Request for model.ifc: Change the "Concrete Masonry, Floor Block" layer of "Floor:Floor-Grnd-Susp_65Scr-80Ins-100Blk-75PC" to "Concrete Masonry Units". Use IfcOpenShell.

First a look at what the model holds.

```python
import ifcopenshell
import ifcopenshell.util.element

model = ifcopenshell.open("model.ifc")
print(model.schema)
for layer_set in model.by_type("IfcMaterialLayerSet"):
    if layer_set.LayerSetName == "Floor:Floor-Grnd-Susp_65Scr-80Ins-100Blk-75PC":
        for layer in layer_set.MaterialLayers:
            print(layer.id(), layer.Material and layer.Material.Name, layer.LayerThickness, sep=" | ")
        print(len(ifcopenshell.util.element.get_elements_by_material(model, layer_set)), "elements and types use it")
print(sorted(m.Name for m in model.by_type("IfcMaterial") if m.Name)[:60])
```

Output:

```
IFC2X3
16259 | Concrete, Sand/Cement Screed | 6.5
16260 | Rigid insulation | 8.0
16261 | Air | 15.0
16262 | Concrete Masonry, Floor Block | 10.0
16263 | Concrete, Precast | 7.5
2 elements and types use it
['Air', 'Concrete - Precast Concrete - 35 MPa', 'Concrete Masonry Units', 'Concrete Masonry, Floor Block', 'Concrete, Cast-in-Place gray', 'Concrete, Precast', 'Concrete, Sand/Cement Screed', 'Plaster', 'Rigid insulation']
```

```python
import ifcopenshell
import ifcopenshell.api.material

model = ifcopenshell.open("model.ifc")

layer_set = next(s for s in model.by_type("IfcMaterialLayerSet") if s.LayerSetName == "Floor:Floor-Grnd-Susp_65Scr-80Ins-100Blk-75PC")
layer = next(l for l in layer_set.MaterialLayers if l.Material and l.Material.Name == "Concrete Masonry, Floor Block")
material = next(m for m in model.by_type("IfcMaterial") if m.Name == "Concrete Masonry Units")

# Point this one layer at the other material; renaming the old one would change it everywhere.
ifcopenshell.api.material.edit_layer(model, layer=layer, attributes={}, material=material)

print([l.Material.Name if l.Material else None for l in layer_set.MaterialLayers])

model.write("model_updated.ifc")
```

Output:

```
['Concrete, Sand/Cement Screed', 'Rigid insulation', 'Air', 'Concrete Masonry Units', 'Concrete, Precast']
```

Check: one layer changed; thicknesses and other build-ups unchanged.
